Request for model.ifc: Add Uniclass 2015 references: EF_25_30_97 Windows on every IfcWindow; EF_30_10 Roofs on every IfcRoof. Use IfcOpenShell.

First a look at what the model holds.

```python
import ifcopenshell

model = ifcopenshell.open("model.ifc")
print(model.schema)
print("classifications:", [c.Name for c in model.by_type("IfcClassification")])
for ifc_class in ("IfcDoor", "IfcRoof", "IfcStair", "IfcWall", "IfcWindow"):
    print(ifc_class, len(model.by_type(ifc_class)))
```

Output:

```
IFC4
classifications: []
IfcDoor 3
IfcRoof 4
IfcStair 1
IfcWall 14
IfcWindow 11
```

```python
import ifcopenshell
import ifcopenshell.api.classification

model = ifcopenshell.open("model.ifc")

system = ifcopenshell.api.classification.add_classification(model, classification="Uniclass 2015")

codes = {
    "IfcWindow": ("EF_25_30_97", "Windows"),
    "IfcRoof": ("EF_30_10", "Roofs"),
}
for ifc_class, (code, name) in codes.items():
    products = model.by_type(ifc_class)
    ifcopenshell.api.classification.add_reference(
        model, products=products, classification=system, identification=code, name=name
    )
    print(code, len(products))

model.write("model_rev.ifc")
```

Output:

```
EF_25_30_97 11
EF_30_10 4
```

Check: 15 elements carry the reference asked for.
